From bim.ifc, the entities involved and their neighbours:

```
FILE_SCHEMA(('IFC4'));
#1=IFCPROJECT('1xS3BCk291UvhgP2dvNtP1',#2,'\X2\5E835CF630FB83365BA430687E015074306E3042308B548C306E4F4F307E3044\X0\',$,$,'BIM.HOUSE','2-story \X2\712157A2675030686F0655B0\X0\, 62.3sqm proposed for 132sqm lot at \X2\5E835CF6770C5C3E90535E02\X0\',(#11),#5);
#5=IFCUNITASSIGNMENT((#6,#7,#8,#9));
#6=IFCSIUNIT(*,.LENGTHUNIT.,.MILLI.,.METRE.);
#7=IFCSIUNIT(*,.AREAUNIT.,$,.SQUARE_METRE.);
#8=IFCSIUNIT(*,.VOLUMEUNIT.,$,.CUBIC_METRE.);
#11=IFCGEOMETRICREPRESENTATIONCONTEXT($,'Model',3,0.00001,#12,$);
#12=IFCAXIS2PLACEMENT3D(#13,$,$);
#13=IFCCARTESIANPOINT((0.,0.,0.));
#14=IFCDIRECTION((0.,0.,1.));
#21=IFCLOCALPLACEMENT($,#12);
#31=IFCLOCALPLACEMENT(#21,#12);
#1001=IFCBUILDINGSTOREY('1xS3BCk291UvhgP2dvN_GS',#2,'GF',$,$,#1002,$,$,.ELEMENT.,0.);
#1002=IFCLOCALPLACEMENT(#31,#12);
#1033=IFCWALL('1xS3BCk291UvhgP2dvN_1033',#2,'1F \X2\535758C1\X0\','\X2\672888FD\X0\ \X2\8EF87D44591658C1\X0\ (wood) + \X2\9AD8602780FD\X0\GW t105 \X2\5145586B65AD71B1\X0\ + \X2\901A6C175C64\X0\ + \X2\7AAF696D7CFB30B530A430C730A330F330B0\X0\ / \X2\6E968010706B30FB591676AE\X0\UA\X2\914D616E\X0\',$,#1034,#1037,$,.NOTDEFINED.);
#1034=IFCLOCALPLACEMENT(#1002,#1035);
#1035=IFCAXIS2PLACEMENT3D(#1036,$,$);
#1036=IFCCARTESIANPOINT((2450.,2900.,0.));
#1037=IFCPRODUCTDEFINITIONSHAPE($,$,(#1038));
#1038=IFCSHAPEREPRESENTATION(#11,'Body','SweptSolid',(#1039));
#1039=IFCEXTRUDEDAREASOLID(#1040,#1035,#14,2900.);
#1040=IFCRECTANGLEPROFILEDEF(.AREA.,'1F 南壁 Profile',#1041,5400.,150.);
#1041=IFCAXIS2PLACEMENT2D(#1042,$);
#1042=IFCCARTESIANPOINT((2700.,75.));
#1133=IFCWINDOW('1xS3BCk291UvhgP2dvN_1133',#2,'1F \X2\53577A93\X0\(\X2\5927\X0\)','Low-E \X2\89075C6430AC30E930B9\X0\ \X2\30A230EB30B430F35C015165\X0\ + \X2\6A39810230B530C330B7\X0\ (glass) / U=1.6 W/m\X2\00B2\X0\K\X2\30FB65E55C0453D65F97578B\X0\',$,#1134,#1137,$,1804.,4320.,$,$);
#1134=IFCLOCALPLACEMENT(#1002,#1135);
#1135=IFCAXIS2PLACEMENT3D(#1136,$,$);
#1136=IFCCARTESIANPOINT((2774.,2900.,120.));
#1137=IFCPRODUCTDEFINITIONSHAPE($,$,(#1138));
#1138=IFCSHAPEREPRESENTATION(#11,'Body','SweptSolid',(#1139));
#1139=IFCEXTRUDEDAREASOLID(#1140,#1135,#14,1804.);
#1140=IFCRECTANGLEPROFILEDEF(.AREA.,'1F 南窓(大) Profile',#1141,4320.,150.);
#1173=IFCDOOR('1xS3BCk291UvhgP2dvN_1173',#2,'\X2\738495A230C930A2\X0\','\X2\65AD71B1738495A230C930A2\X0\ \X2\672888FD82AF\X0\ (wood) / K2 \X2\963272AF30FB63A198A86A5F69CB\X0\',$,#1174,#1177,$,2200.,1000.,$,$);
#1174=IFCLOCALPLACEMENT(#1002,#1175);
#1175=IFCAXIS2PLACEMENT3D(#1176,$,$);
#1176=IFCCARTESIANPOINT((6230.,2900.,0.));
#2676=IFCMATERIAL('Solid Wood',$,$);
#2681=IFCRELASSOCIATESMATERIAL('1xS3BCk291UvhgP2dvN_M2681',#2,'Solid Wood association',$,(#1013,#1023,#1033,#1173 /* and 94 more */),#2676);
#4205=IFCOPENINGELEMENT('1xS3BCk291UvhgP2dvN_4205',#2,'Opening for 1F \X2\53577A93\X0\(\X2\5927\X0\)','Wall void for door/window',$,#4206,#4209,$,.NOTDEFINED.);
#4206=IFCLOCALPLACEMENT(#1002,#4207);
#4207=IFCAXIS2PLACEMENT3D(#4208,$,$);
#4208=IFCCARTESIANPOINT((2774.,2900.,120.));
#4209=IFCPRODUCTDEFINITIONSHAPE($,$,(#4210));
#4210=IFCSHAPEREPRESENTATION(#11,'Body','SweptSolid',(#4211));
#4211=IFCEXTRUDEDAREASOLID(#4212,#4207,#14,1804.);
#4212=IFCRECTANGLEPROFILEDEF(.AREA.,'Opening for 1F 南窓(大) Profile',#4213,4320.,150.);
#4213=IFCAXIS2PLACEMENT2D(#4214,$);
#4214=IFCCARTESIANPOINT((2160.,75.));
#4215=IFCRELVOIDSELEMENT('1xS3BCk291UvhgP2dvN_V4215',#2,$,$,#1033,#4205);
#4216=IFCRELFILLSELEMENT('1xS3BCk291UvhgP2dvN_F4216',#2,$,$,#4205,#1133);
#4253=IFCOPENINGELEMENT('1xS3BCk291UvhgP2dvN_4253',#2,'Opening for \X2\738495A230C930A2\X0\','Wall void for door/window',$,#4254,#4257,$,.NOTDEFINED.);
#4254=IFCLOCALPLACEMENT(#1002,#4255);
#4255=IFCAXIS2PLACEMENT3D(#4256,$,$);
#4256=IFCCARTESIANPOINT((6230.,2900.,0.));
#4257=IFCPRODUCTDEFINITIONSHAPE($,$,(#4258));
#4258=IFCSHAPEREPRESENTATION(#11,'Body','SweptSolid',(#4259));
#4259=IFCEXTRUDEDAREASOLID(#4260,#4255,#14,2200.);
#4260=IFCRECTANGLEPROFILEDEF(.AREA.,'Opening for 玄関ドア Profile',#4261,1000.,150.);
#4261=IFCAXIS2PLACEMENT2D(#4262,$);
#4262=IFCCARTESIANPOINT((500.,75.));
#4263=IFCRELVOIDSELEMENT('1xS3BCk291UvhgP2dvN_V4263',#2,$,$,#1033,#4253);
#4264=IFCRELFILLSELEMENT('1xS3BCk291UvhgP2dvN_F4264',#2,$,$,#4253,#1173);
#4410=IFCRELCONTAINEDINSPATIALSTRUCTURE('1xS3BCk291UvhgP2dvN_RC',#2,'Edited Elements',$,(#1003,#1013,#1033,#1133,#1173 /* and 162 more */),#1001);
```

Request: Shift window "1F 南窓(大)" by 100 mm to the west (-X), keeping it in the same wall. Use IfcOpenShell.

```python
import ifcopenshell
import ifcopenshell.api.geometry
import ifcopenshell.util.placement

model = ifcopenshell.open("bim.ifc")

window = model.by_id(1133)
opening = window.FillsVoids[0].RelatingOpeningElement
wall = opening.VoidsElements[0].RelatingBuildingElement

wall_matrix = ifcopenshell.util.placement.get_local_placement(wall.ObjectPlacement)
shift = wall_matrix[:3, 0] * -100.0
before = ifcopenshell.util.placement.get_local_placement(window.ObjectPlacement)[:3, 3].copy()

# The window is not placed relative to its opening, so move both.
for product in (opening, window):
    matrix = ifcopenshell.util.placement.get_local_placement(product.ObjectPlacement)
    matrix[:3, 3] += shift
    ifcopenshell.api.geometry.edit_object_placement(model, product=product, matrix=matrix, is_si=False)

after = ifcopenshell.util.placement.get_local_placement(window.ObjectPlacement)[:3, 3]
print("window moved by", (after - before).round(3) + 0.0)

model.write("bim_edited.ifc")
```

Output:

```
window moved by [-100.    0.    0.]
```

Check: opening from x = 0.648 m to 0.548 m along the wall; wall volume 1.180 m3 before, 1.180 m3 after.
